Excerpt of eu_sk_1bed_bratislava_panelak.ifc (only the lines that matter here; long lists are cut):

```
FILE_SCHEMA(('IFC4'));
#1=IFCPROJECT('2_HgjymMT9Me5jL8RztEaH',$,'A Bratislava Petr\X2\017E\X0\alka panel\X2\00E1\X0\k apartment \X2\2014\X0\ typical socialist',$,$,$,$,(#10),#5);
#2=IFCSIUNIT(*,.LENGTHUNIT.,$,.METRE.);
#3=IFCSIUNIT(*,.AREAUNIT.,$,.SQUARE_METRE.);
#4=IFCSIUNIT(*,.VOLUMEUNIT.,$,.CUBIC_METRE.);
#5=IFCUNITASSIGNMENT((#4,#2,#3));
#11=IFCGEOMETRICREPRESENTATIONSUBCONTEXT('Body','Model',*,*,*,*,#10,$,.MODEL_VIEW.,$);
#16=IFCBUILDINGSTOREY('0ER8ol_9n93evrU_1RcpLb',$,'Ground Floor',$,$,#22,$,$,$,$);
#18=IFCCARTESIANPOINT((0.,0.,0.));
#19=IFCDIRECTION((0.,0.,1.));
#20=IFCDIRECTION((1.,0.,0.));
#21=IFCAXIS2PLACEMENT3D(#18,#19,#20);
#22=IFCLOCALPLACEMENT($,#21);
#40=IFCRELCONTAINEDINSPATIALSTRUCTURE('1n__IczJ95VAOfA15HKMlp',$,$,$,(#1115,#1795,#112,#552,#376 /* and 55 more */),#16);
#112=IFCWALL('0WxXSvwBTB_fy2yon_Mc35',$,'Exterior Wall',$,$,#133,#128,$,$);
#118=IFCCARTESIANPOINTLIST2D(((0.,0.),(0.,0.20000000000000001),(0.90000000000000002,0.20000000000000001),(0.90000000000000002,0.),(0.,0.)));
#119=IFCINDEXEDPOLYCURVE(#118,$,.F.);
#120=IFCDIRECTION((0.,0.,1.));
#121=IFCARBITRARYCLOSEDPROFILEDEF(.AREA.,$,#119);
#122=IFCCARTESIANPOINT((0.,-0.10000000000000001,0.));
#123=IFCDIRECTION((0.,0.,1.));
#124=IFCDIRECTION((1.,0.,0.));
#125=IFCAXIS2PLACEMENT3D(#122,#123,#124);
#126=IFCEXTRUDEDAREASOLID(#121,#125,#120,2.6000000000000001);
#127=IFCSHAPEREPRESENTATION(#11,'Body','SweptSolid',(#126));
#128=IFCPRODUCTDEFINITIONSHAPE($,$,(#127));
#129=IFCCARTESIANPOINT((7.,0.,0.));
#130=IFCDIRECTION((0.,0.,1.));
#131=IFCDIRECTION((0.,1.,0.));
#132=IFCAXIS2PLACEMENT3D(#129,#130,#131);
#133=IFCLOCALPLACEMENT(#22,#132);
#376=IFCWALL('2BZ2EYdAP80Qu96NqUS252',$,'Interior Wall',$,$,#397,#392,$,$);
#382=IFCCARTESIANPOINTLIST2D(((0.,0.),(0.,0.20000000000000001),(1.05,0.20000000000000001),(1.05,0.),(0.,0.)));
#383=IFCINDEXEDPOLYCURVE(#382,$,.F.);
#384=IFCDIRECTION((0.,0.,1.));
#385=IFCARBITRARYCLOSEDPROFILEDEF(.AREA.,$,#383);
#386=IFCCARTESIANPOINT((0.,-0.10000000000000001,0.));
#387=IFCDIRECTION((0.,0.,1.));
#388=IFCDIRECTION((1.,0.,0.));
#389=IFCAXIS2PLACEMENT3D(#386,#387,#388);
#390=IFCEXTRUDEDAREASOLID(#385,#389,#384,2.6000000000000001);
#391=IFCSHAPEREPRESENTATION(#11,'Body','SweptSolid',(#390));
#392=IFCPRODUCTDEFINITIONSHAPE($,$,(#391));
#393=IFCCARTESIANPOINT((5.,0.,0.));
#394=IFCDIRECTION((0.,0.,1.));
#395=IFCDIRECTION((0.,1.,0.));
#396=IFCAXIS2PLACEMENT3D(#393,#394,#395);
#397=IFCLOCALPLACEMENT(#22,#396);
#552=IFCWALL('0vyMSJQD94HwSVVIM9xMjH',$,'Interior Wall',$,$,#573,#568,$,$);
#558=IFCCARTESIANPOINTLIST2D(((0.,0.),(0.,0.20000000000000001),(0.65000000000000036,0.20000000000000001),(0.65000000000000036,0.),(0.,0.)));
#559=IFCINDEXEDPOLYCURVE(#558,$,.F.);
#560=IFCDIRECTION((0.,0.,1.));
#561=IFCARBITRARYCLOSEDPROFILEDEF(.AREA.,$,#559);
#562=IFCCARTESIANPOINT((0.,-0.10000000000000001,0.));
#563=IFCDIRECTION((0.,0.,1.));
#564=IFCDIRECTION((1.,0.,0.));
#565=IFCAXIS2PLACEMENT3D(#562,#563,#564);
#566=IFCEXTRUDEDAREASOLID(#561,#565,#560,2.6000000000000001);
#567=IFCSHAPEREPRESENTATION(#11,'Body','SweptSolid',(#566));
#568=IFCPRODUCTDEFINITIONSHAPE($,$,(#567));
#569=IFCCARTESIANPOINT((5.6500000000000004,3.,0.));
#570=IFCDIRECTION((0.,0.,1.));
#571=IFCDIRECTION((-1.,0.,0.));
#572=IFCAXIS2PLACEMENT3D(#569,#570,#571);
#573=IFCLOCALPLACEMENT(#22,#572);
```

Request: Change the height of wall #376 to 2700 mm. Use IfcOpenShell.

```python
import ifcopenshell
import ifcopenshell.geom
import ifcopenshell.util.representation
import ifcopenshell.util.shape
import ifcopenshell.util.unit

model = ifcopenshell.open("eu_sk_1bed_bratislava_panelak.ifc")
unit_scale = ifcopenshell.util.unit.calculate_unit_scale(model)
settings = ifcopenshell.geom.settings()


def volume(element):
    """Net volume in cubic metres, openings subtracted."""
    shape = ifcopenshell.geom.create_shape(settings, element)
    return ifcopenshell.util.shape.get_volume(shape.geometry)


wall = model.by_guid("2BZ2EYdAP80Qu96NqUS252")
before = volume(wall)

body = ifcopenshell.util.representation.get_representation(wall, "Model", "Body")
solid = body.Items[0]
old_height = solid.Depth
solid.Depth = 2.7 / unit_scale
after = volume(wall)

print(f"height {old_height:g} -> {solid.Depth:g}, volume {before:.3f} -> {after:.3f} m3")

model.write("eu_sk_1bed_bratislava_panelak_rev.ifc")
```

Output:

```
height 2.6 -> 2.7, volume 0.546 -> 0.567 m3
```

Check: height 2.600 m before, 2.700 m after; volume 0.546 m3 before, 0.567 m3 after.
